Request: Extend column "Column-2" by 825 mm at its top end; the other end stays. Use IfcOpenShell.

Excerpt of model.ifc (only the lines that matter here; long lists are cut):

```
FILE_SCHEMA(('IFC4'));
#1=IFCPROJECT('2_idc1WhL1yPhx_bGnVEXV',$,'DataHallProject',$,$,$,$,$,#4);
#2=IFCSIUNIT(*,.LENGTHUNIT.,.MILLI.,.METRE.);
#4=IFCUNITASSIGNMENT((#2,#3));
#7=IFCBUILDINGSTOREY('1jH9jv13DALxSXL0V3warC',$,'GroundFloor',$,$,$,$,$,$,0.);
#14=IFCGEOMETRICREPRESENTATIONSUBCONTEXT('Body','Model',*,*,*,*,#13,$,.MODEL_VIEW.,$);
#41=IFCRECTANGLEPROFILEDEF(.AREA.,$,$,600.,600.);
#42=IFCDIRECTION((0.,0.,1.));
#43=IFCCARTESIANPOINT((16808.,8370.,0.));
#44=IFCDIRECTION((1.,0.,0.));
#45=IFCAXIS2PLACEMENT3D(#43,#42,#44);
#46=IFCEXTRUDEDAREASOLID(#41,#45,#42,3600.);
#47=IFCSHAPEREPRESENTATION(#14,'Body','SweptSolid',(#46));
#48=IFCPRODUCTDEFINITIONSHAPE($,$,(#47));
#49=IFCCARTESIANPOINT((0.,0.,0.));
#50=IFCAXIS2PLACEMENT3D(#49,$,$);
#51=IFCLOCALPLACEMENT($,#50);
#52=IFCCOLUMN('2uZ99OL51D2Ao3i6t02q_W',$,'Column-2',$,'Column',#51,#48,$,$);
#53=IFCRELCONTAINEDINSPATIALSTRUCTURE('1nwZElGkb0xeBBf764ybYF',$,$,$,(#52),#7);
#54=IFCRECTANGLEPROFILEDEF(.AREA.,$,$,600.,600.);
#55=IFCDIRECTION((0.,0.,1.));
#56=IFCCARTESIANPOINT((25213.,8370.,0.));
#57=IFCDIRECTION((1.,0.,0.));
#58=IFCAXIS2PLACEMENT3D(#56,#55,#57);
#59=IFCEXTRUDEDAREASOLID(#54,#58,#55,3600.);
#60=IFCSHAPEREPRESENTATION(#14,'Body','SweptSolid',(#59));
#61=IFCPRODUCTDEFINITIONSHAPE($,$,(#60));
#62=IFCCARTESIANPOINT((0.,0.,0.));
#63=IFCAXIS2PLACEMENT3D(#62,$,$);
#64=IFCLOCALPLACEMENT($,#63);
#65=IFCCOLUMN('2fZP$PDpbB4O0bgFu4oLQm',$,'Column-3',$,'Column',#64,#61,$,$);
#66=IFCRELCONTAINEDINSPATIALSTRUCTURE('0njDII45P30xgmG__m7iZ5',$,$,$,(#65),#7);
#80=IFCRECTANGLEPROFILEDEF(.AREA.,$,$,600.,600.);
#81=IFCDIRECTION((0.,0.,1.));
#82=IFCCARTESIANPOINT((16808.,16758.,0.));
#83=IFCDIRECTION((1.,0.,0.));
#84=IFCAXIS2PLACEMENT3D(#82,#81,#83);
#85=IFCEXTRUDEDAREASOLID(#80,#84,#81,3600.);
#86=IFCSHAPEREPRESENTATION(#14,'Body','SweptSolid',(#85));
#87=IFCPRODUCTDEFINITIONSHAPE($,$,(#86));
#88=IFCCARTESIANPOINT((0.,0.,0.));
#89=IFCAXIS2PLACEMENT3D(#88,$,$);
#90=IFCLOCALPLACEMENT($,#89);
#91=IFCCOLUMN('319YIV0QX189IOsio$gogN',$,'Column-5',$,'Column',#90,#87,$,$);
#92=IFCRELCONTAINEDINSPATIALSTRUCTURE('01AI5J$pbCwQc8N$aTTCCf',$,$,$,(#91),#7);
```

```python
import ifcopenshell
import ifcopenshell.util.representation

model = ifcopenshell.open("model.ifc")

member = model.by_guid("2uZ99OL51D2Ao3i6t02q_W")
change = 825.0

# The extrusion runs towards the end named, so only its depth changes.
body = ifcopenshell.util.representation.get_representation(member, "Model", "Body")
solid = body.Items[0]
old_length = solid.Depth
solid.Depth += change

print(f"length {old_length:g} -> {solid.Depth:g}")

model.write("model_rev.ifc")
```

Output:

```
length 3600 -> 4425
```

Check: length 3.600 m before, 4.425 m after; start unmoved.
